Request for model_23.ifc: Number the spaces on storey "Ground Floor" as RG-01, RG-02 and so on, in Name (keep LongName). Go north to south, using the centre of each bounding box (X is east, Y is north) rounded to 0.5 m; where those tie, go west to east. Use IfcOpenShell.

First a look at what the model holds.

```python
import ifcopenshell
import ifcopenshell.util.element
import ifcopenshell.util.placement

model = ifcopenshell.open("model_23.ifc")
print(model.schema)
storey = next(s for s in model.by_type("IfcBuildingStorey") if s.Name == "Ground Floor")
spaces = [e for e in ifcopenshell.util.element.get_decomposition(storey) if e.is_a("IfcSpace")]
for e in sorted(spaces, key=lambda e: e.id()):
    origin = ifcopenshell.util.placement.get_local_placement(e.ObjectPlacement)[:3, 3]
    print(e.id(), e.Name, e.LongName, origin.round(2) + 0.0, sep=" | ")
```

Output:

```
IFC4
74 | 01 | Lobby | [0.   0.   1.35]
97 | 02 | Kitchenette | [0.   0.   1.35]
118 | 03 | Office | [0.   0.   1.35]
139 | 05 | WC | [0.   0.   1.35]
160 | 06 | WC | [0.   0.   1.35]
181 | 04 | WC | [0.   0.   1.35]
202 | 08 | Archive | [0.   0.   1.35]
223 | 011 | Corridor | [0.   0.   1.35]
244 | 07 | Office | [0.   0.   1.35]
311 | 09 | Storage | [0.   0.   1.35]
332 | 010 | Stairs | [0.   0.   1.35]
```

```python
import ifcopenshell
import ifcopenshell.geom
import ifcopenshell.util.element
import ifcopenshell.util.shape

model = ifcopenshell.open("model_23.ifc")
settings = ifcopenshell.geom.settings()
settings.set("use-world-coords", True)


def centre(element):
    shape = ifcopenshell.geom.create_shape(settings, element)
    return ifcopenshell.util.shape.get_bbox_centroid(shape.geometry)


storey = next(s for s in model.by_type("IfcBuildingStorey") if s.Name == "Ground Floor")
spaces = [e for e in ifcopenshell.util.element.get_decomposition(storey) if e.is_a("IfcSpace")]

# Insertion points can sit at a corner or the storey origin, so sort by the geometry (in metres).
centres = {e: centre(e) for e in spaces}
spaces.sort(key=lambda e: (-round(centres[e][1] / 0.5), centres[e][0]))

for i, e in enumerate(spaces, start=1):
    number = f"RG-{i:02d}"
    e.Name = number
    print(e.id(), number)

model.write("model_23_rev.ifc")
```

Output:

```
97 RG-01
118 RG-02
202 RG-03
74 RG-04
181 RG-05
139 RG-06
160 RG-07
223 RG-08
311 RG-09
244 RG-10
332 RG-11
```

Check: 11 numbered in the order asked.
